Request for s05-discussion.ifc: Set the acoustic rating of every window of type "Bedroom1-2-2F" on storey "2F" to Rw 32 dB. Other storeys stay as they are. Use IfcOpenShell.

First a look at what the model holds.

```python
import ifcopenshell
import ifcopenshell.util.element

model = ifcopenshell.open("s05-discussion.ifc")
print(model.schema)
storey = next(s for s in model.by_type("IfcBuildingStorey") if s.Name == "2F")
windows = [e for e in ifcopenshell.util.element.get_decomposition(storey) if e.is_a("IfcWindow")]
seen = {}
for e in windows:
    element_type = ifcopenshell.util.element.get_type(e)
    key = (element_type.Name if element_type != e and element_type else None, ifcopenshell.util.element.get_pset(e, "Pset_WindowCommon", "AcousticRating"))
    seen[key] = seen.get(key, 0) + 1
for (name, value), count in sorted(seen.items(), key=str):
    print(count, "x", name, "|", value)
```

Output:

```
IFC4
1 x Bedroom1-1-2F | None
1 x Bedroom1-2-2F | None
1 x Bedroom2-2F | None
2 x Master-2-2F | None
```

```python
import ifcopenshell
import ifcopenshell.api.pset
import ifcopenshell.util.element

model = ifcopenshell.open("s05-discussion.ifc")

storey = next(s for s in model.by_type("IfcBuildingStorey") if s.Name == "2F")
windows = [e for e in ifcopenshell.util.element.get_decomposition(storey) if e.is_a("IfcWindow")]

count = 0
for e in windows:
    element_type = ifcopenshell.util.element.get_type(e)
    if element_type in (None, e) or element_type.Name != "Bedroom1-2-2F":
        continue
    # add_pset returns the element's existing set when there is one.
    pset = ifcopenshell.api.pset.add_pset(model, product=e, name="Pset_WindowCommon")
    ifcopenshell.api.pset.edit_pset(model, pset=pset, properties={"AcousticRating": "Rw 32 dB"})
    count += 1

print(count, "windows updated")

model.write("s05-discussion_edited.ifc")
```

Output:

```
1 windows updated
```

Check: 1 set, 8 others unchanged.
